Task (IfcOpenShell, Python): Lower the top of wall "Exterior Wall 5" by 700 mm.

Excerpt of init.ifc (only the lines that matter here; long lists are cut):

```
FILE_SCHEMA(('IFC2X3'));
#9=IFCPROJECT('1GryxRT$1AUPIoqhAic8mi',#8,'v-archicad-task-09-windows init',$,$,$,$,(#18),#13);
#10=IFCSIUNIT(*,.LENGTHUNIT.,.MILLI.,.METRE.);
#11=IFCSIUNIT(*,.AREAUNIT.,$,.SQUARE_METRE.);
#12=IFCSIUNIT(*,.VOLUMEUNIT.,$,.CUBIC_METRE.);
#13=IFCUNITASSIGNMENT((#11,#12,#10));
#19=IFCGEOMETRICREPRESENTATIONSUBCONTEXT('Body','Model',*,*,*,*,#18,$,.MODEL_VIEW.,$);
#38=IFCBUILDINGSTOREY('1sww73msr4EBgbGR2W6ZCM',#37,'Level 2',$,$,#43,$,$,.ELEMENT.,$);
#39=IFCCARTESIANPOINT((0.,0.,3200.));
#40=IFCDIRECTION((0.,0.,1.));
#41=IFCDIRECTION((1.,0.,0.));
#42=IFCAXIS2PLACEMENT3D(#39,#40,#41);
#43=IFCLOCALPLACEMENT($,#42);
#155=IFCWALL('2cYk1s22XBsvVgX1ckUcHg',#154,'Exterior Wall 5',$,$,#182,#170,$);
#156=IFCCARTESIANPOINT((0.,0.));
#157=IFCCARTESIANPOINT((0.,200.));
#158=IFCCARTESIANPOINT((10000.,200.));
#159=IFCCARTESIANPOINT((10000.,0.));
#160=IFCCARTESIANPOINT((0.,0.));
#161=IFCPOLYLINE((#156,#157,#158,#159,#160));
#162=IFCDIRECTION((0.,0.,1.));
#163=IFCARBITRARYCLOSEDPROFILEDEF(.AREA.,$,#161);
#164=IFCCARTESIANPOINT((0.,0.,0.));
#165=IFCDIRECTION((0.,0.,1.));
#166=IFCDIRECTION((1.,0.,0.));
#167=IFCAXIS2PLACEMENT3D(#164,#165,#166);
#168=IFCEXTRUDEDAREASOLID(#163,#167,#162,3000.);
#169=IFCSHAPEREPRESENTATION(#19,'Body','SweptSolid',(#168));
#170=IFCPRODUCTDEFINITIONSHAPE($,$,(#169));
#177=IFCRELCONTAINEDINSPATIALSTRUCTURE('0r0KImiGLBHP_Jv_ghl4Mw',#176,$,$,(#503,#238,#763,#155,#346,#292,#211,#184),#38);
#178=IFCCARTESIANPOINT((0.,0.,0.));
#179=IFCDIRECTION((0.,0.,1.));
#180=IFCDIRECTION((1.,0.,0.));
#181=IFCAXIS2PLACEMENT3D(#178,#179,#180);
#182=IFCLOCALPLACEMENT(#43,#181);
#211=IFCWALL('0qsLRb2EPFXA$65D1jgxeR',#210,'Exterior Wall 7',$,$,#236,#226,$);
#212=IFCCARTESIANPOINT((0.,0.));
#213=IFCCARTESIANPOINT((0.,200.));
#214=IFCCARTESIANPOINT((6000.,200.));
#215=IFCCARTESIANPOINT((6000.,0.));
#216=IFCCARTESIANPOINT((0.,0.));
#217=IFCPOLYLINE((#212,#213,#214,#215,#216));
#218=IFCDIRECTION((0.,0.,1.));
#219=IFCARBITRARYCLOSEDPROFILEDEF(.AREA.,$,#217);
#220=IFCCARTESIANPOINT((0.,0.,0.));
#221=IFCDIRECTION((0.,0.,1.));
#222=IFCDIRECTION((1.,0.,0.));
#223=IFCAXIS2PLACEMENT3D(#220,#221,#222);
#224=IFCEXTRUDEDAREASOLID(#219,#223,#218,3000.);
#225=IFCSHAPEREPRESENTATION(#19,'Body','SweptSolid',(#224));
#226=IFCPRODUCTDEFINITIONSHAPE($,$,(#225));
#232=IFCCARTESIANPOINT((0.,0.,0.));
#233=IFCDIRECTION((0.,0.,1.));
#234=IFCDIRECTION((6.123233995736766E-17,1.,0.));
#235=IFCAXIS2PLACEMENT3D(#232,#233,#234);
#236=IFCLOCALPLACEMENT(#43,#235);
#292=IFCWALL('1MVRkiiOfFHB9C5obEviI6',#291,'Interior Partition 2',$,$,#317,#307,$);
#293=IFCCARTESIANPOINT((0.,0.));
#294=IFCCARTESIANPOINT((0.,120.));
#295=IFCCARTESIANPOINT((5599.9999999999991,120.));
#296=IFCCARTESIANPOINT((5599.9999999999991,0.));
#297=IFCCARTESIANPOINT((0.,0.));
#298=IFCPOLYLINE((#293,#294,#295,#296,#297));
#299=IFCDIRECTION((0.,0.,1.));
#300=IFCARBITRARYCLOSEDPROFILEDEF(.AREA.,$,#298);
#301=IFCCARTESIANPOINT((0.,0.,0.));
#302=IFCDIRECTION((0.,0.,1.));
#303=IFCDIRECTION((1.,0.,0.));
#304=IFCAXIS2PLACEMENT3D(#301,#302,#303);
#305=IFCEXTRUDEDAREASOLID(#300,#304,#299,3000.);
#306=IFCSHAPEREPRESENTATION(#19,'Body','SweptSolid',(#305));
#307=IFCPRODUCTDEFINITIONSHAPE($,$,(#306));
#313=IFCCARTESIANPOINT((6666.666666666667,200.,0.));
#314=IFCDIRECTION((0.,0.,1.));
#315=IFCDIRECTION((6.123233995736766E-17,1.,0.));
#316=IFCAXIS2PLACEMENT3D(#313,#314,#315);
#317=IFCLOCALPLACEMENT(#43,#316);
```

```python
import ifcopenshell
import ifcopenshell.geom
import ifcopenshell.util.representation
import ifcopenshell.util.shape
import ifcopenshell.util.unit

model = ifcopenshell.open("init.ifc")
unit_scale = ifcopenshell.util.unit.calculate_unit_scale(model)
settings = ifcopenshell.geom.settings()


def volume(element):
    """Net volume in cubic metres, openings subtracted."""
    shape = ifcopenshell.geom.create_shape(settings, element)
    return ifcopenshell.util.shape.get_volume(shape.geometry)


wall = model.by_guid("2cYk1s22XBsvVgX1ckUcHg")
before = volume(wall)

body = ifcopenshell.util.representation.get_representation(wall, "Model", "Body")
solid = body.Items[0]
old_height = solid.Depth
solid.Depth -= 0.7 / unit_scale
after = volume(wall)

print(f"height {old_height:g} -> {solid.Depth:g}, volume {before:.3f} -> {after:.3f} m3")

model.write("init_v2.ifc")
```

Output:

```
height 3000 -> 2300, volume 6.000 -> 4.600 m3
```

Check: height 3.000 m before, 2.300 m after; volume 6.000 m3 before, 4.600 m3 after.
